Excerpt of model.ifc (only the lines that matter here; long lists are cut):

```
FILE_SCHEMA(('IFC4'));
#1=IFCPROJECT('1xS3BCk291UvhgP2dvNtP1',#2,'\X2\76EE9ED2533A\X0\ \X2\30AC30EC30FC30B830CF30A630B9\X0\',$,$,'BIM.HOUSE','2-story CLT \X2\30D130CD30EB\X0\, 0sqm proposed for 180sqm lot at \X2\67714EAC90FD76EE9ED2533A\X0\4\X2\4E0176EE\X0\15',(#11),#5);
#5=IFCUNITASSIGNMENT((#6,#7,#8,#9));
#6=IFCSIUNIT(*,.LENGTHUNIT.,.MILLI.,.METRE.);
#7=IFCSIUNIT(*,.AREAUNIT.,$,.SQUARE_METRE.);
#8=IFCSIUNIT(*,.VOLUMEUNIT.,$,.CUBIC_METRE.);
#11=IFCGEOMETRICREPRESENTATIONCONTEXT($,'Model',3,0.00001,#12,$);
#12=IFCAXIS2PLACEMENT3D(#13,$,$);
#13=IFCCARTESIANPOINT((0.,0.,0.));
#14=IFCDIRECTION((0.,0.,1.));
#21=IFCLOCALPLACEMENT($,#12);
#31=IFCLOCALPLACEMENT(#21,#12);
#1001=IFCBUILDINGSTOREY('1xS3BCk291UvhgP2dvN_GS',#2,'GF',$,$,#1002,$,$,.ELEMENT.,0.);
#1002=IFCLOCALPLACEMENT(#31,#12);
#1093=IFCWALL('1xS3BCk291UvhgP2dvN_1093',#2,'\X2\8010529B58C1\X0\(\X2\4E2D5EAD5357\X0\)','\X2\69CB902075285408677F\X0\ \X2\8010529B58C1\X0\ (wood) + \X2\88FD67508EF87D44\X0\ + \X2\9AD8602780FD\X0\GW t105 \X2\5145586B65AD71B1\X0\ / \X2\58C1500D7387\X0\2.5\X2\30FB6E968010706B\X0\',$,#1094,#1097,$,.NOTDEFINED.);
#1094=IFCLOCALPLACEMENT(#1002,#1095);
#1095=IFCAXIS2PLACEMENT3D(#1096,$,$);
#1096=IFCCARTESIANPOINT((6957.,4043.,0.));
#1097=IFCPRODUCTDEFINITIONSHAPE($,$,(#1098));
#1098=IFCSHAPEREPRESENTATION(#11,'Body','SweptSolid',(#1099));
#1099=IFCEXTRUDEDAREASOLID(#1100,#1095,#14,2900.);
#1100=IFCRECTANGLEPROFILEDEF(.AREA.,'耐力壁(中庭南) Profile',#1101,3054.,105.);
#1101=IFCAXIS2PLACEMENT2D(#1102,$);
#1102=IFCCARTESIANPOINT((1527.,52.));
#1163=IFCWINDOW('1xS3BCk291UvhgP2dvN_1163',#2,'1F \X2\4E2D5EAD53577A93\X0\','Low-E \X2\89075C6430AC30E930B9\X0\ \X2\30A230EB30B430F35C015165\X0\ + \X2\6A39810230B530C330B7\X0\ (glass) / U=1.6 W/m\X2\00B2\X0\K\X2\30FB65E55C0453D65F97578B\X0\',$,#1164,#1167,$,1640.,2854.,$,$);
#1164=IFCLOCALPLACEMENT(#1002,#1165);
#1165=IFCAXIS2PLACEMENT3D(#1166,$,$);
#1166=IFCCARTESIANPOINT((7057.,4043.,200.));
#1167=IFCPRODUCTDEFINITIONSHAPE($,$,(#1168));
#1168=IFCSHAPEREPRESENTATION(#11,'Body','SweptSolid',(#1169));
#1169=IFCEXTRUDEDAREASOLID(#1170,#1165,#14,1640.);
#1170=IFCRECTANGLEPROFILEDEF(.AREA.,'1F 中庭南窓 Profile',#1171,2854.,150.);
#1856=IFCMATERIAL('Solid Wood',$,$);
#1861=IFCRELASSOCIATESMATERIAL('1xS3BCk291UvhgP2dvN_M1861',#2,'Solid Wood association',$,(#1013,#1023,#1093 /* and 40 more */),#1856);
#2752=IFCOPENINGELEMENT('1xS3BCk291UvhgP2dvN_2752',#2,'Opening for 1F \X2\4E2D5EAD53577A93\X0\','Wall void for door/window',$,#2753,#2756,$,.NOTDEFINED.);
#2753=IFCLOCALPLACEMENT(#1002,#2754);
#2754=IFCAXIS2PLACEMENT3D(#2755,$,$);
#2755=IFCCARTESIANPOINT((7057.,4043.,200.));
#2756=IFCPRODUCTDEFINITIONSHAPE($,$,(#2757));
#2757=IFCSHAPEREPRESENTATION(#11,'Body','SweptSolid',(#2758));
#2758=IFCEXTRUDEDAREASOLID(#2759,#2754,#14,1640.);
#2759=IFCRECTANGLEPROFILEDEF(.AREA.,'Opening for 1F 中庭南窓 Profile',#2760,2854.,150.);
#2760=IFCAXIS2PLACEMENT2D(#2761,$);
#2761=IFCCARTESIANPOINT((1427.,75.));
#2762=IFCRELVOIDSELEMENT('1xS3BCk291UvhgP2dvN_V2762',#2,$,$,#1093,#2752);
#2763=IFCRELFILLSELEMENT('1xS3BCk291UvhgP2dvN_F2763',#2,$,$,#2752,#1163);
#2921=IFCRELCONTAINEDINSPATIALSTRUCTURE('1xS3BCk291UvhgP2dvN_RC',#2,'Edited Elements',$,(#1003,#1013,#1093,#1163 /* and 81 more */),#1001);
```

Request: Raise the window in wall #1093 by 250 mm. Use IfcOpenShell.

```python
import numpy as np
import ifcopenshell
import ifcopenshell.api.geometry
import ifcopenshell.util.placement
import ifcopenshell.util.unit

model = ifcopenshell.open("model.ifc")
unit_scale = ifcopenshell.util.unit.calculate_unit_scale(model)

window = model.by_guid("1xS3BCk291UvhgP2dvN_1163")
opening = window.FillsVoids[0].RelatingOpeningElement
dz = 0.25 / unit_scale

shift = np.array([0.0, 0.0, dz])
# The window is not placed relative to its opening, so move both.
for product in (opening, window):
    matrix = ifcopenshell.util.placement.get_local_placement(product.ObjectPlacement)
    matrix[:3, 3] += shift
    ifcopenshell.api.geometry.edit_object_placement(model, product=product, matrix=matrix, is_si=False)

print(f"moved by {dz * unit_scale:+.3f} m")

model.write("model_v2.ifc")
```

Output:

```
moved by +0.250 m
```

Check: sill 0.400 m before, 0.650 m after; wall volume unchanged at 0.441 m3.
